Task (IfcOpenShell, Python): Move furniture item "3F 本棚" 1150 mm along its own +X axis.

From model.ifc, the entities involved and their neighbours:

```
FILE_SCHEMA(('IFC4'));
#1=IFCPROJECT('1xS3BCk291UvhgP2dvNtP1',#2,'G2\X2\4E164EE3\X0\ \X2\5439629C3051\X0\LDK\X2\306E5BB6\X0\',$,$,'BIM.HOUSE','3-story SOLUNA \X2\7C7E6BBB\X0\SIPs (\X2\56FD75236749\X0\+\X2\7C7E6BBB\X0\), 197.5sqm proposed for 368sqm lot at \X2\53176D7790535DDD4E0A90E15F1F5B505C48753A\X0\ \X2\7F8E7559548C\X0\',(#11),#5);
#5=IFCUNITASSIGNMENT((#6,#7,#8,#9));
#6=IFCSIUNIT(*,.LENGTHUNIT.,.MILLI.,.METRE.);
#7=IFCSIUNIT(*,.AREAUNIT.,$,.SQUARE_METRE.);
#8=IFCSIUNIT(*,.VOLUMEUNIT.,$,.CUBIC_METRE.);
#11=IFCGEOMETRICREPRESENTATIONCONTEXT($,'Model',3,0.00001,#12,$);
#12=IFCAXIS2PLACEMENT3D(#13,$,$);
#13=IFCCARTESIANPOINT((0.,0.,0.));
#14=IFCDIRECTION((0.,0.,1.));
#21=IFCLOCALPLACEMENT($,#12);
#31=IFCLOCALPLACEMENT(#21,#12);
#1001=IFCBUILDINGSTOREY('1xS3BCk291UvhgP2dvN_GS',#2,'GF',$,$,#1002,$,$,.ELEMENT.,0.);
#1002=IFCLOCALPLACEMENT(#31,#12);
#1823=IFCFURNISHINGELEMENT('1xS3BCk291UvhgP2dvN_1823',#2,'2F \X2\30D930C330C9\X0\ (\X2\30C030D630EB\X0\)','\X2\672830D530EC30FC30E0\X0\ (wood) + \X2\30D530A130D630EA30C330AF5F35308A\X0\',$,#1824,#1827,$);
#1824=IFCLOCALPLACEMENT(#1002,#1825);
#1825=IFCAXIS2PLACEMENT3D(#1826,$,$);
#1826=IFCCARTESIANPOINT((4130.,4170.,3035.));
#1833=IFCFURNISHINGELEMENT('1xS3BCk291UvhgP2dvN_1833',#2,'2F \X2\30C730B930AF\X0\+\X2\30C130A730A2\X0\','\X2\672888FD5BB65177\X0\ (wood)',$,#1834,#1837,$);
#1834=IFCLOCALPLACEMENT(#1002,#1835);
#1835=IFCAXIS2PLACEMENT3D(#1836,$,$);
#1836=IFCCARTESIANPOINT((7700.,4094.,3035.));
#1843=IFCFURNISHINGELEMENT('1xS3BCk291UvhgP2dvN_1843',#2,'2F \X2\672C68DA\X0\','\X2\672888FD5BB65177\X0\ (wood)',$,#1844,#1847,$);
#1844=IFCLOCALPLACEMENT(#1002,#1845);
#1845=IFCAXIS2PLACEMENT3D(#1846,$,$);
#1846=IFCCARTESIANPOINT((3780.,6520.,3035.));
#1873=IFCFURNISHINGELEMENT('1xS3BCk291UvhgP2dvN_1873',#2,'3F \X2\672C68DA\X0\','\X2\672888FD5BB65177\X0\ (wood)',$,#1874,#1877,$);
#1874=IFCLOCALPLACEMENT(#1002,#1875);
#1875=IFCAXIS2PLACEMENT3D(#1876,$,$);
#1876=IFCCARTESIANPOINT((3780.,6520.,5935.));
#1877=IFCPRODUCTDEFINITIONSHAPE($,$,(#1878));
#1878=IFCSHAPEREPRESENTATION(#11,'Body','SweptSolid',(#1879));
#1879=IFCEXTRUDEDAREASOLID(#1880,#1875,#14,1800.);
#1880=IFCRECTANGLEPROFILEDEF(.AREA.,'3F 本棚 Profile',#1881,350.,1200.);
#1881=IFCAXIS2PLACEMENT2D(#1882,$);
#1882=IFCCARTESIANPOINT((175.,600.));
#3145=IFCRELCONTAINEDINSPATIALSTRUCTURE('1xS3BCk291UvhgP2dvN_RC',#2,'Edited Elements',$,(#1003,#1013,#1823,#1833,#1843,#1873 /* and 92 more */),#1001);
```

```python
import ifcopenshell
import ifcopenshell.api.geometry
import ifcopenshell.util.placement
import ifcopenshell.util.unit

model = ifcopenshell.open("model.ifc")
unit_scale = ifcopenshell.util.unit.calculate_unit_scale(model)

item = model.by_guid("1xS3BCk291UvhgP2dvN_1873")
matrix = ifcopenshell.util.placement.get_local_placement(item.ObjectPlacement)
matrix[:3, 3] += matrix[:3, 0] * 1.15 / unit_scale
ifcopenshell.api.geometry.edit_object_placement(model, product=item, matrix=matrix, is_si=False)

print(ifcopenshell.util.placement.get_local_placement(item.ObjectPlacement).round(3) + 0.0)

model.write("model_rev.ifc")
```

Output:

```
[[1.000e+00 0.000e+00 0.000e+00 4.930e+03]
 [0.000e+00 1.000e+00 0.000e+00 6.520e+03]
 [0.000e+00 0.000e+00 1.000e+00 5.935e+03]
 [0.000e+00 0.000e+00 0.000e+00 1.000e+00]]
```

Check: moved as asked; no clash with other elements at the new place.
